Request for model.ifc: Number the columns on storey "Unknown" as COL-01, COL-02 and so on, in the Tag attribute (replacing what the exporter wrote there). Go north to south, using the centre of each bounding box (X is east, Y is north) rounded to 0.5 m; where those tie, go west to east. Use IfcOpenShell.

First a look at what the model holds.

```python
import ifcopenshell
import ifcopenshell.util.element
import ifcopenshell.util.placement

model = ifcopenshell.open("model.ifc")
print(model.schema)
storey = next(s for s in model.by_type("IfcBuildingStorey") if s.Name == "Unknown")
columns = [e for e in ifcopenshell.util.element.get_decomposition(storey) if e.is_a("IfcColumn")]
for e in sorted(columns, key=lambda e: e.id()):
    origin = ifcopenshell.util.placement.get_local_placement(e.ObjectPlacement)[:3, 3]
    print(e.id(), e.Tag, e.Name, origin.round(2) + 0.0, sep=" | ")
```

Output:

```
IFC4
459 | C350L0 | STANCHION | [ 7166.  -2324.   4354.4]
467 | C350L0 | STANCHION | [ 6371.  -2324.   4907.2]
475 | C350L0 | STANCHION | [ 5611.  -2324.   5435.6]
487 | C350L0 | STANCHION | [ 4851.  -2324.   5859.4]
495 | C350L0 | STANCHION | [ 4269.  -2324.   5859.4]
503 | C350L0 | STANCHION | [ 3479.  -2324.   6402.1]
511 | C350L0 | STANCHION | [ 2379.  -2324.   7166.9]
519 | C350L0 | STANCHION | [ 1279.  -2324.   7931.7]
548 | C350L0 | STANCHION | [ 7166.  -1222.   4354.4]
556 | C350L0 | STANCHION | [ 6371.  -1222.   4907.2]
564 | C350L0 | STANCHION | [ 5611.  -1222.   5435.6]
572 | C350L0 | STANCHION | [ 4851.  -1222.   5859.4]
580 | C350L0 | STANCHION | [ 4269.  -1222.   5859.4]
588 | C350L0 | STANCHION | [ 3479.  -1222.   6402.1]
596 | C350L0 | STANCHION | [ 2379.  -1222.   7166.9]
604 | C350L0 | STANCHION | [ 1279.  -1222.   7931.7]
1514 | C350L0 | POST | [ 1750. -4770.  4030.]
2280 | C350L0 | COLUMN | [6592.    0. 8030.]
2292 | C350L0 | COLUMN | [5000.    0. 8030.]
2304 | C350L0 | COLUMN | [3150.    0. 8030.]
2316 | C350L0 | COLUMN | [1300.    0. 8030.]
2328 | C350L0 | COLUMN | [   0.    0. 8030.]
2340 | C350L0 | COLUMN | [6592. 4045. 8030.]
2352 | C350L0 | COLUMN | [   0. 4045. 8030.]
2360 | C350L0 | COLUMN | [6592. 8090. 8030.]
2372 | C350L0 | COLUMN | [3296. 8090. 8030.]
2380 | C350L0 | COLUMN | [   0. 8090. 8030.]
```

```python
import ifcopenshell
import ifcopenshell.geom
import ifcopenshell.util.element
import ifcopenshell.util.shape

model = ifcopenshell.open("model.ifc")
settings = ifcopenshell.geom.settings()
settings.set("use-world-coords", True)


def centre(element):
    shape = ifcopenshell.geom.create_shape(settings, element)
    return ifcopenshell.util.shape.get_bbox_centroid(shape.geometry)


storey = next(s for s in model.by_type("IfcBuildingStorey") if s.Name == "Unknown")
columns = [e for e in ifcopenshell.util.element.get_decomposition(storey) if e.is_a("IfcColumn")]

# Insertion points can sit at a corner or the storey origin, so sort by the geometry (in metres).
centres = {e: centre(e) for e in columns}
columns.sort(key=lambda e: (-round(centres[e][1] / 0.5), centres[e][0]))

for i, e in enumerate(columns, start=1):
    number = f"COL-{i:02d}"
    e.Tag = number
    print(e.id(), number)

model.write("model_v2.ifc")
```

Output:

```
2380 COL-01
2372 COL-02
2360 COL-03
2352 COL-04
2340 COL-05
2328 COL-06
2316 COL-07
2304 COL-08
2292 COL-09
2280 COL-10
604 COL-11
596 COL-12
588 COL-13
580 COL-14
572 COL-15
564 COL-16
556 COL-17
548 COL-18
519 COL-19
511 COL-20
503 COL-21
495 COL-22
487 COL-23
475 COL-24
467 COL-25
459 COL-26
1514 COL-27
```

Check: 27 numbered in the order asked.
